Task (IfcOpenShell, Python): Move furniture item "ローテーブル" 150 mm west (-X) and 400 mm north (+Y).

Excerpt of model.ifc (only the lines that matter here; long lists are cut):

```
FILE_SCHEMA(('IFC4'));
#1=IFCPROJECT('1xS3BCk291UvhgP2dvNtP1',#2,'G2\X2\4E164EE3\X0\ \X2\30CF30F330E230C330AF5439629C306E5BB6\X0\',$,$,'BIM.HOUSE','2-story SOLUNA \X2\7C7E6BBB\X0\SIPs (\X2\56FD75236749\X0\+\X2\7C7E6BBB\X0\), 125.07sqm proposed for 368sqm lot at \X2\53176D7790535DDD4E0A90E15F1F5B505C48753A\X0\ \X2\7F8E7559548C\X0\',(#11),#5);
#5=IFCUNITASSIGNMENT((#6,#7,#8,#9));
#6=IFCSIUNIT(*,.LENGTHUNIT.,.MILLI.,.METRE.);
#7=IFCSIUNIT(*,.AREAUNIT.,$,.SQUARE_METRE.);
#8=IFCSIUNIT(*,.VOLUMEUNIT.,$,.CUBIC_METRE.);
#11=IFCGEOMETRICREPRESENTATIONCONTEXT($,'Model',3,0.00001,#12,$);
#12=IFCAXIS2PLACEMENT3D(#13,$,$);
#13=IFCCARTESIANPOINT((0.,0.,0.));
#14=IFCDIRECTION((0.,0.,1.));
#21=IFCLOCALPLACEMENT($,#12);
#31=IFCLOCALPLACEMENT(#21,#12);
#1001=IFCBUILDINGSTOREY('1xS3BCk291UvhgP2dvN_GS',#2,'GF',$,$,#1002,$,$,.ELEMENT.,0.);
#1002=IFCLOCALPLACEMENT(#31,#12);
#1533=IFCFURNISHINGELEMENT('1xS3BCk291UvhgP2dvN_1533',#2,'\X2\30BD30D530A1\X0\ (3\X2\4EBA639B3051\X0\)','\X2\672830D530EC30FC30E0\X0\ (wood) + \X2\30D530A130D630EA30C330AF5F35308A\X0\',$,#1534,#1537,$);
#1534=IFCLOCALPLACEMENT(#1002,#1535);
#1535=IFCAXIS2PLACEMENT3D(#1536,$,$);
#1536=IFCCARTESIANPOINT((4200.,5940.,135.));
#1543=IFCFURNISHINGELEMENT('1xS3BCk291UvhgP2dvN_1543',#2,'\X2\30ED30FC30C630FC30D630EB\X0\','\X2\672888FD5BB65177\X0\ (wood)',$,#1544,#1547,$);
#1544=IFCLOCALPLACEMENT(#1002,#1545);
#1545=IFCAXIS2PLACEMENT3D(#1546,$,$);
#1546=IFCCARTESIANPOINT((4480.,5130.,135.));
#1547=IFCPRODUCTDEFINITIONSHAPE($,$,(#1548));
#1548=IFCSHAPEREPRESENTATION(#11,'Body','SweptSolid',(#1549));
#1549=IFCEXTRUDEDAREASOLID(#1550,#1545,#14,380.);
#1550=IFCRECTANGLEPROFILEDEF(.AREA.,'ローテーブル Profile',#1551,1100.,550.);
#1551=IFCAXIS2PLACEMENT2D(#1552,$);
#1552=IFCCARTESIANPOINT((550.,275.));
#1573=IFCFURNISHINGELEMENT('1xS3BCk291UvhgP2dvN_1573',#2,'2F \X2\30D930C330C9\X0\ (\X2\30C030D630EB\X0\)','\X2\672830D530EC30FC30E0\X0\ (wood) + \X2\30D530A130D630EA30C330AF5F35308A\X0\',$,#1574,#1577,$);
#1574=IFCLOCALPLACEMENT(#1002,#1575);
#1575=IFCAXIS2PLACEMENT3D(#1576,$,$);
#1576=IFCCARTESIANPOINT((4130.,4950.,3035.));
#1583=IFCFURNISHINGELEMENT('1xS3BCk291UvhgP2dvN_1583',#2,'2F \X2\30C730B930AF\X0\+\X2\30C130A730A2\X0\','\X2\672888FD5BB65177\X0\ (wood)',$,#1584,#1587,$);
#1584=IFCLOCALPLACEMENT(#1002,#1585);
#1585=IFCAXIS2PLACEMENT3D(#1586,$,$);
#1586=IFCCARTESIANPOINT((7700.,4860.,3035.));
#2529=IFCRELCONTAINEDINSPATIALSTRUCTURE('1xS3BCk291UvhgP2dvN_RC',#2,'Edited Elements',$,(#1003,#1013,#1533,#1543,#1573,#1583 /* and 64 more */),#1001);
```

```python
import ifcopenshell
import ifcopenshell.api.geometry
import ifcopenshell.util.placement
import ifcopenshell.util.unit

model = ifcopenshell.open("model.ifc")
unit_scale = ifcopenshell.util.unit.calculate_unit_scale(model)

item = model.by_id(1543)
matrix = ifcopenshell.util.placement.get_local_placement(item.ObjectPlacement)
matrix[0, 3] -= 0.15 / unit_scale
matrix[1, 3] += 0.4 / unit_scale
ifcopenshell.api.geometry.edit_object_placement(model, product=item, matrix=matrix, is_si=False)

print(ifcopenshell.util.placement.get_local_placement(item.ObjectPlacement).round(3) + 0.0)

model.write("model-out.ifc")
```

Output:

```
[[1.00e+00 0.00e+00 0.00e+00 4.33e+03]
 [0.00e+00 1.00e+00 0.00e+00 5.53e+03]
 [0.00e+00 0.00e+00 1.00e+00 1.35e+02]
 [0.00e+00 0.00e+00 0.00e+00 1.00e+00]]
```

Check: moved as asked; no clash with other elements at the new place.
